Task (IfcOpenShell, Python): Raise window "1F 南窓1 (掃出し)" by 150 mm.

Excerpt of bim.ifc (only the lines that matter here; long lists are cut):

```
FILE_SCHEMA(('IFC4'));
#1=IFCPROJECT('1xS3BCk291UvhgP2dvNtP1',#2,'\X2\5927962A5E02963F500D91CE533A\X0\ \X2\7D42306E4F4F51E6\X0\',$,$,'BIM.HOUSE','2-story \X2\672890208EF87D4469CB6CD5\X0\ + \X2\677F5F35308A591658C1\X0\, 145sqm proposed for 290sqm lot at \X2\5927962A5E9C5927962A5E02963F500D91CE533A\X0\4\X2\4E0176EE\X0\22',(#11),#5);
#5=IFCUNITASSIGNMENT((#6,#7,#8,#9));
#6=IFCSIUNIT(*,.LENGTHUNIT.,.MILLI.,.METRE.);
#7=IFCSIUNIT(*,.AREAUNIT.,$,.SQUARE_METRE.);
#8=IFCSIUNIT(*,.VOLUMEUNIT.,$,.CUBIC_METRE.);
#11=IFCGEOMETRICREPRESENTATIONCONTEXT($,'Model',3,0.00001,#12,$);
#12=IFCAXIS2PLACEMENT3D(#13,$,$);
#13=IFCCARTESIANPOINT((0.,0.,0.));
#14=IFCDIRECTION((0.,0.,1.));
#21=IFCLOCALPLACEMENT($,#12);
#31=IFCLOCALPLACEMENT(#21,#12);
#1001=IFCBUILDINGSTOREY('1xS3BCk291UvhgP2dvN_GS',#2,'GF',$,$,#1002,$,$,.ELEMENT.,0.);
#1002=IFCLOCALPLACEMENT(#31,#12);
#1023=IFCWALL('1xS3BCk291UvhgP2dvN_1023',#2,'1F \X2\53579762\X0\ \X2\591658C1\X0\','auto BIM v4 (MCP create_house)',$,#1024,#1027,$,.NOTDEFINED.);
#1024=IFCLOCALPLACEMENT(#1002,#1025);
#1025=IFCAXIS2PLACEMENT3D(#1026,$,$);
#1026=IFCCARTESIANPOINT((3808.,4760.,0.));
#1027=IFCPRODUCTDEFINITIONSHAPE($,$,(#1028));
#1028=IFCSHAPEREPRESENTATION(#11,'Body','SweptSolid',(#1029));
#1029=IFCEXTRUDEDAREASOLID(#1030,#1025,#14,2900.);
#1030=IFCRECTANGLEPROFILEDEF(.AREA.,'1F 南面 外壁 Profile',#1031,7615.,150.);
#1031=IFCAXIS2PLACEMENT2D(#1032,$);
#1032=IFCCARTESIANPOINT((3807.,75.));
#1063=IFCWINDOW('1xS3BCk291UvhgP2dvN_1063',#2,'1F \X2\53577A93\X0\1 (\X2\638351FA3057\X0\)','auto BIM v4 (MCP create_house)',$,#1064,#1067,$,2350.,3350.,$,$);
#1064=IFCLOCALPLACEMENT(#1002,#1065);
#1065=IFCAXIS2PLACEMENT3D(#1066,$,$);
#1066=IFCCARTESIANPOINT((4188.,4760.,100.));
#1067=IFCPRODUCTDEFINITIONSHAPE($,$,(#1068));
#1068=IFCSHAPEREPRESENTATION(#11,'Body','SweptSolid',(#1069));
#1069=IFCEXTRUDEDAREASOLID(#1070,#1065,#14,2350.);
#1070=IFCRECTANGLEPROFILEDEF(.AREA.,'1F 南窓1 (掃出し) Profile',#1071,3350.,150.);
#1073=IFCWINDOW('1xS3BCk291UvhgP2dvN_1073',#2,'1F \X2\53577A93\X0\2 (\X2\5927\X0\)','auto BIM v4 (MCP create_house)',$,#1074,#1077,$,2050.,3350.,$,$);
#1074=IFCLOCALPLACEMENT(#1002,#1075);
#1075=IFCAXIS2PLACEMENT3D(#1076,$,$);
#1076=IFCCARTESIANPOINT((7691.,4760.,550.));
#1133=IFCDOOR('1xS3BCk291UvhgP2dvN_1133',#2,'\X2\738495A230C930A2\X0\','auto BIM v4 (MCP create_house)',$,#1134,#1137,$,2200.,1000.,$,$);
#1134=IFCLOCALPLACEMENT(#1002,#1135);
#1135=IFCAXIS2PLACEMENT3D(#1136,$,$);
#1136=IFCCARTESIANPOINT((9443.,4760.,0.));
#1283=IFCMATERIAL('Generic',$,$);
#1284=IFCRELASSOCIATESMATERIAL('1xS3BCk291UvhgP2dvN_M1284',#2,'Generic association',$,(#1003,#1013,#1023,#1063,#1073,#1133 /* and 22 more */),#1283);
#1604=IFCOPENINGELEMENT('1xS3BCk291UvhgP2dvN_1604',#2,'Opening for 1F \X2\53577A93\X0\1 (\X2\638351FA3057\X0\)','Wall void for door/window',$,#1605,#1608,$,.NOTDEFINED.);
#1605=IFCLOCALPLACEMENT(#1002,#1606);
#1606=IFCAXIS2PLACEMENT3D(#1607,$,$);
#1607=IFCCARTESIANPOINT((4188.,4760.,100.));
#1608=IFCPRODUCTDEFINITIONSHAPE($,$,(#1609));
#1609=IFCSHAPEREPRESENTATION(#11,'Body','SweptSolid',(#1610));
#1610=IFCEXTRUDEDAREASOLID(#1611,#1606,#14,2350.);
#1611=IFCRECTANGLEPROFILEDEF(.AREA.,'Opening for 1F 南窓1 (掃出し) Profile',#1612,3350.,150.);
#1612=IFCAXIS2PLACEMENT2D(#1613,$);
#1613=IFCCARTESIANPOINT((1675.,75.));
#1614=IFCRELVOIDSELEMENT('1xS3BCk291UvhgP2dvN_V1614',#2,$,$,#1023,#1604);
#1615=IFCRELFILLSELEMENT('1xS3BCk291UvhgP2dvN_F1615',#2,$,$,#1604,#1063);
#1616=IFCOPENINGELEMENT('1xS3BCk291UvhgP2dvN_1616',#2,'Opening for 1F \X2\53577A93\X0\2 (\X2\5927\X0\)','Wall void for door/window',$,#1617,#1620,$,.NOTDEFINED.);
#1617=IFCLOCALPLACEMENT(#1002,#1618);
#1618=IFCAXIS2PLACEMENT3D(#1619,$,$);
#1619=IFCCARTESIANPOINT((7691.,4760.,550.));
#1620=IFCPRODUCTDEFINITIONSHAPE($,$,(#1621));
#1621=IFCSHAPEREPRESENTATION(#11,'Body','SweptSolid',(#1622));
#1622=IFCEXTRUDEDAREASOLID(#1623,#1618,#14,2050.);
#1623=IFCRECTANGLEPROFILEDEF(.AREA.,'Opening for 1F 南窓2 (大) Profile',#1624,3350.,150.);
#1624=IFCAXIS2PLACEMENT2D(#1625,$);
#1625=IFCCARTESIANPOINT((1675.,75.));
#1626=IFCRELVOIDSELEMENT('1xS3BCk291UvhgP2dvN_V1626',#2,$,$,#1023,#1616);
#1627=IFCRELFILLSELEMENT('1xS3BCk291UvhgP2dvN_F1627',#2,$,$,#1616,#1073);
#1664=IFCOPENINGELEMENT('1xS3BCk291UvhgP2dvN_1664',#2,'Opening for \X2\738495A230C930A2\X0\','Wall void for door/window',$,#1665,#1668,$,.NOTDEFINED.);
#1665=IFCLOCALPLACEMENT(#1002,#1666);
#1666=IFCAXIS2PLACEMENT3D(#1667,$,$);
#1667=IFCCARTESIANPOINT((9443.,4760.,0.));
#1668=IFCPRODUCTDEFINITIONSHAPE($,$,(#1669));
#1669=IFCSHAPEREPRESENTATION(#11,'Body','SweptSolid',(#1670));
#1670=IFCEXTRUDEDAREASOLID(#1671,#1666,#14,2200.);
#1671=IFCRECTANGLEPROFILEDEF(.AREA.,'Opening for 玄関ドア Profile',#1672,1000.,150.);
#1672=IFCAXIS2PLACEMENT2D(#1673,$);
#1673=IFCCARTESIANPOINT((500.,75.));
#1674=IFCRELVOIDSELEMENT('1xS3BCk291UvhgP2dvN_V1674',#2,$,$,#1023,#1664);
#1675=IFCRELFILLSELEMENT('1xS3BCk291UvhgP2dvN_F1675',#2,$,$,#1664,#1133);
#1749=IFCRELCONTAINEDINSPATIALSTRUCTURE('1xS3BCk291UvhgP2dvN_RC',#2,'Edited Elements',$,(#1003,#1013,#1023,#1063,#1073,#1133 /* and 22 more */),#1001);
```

```python
import numpy as np
import ifcopenshell
import ifcopenshell.api.geometry
import ifcopenshell.util.placement
import ifcopenshell.util.unit

model = ifcopenshell.open("bim.ifc")
unit_scale = ifcopenshell.util.unit.calculate_unit_scale(model)

window = model.by_id(1063)
opening = window.FillsVoids[0].RelatingOpeningElement
dz = 150.0

shift = np.array([0.0, 0.0, dz])
# The window is not placed relative to its opening, so move both.
for product in (opening, window):
    matrix = ifcopenshell.util.placement.get_local_placement(product.ObjectPlacement)
    matrix[:3, 3] += shift
    ifcopenshell.api.geometry.edit_object_placement(model, product=product, matrix=matrix, is_si=False)

print(f"moved by {dz * unit_scale:+.3f} m")

model.write("bim_edited.ifc")
```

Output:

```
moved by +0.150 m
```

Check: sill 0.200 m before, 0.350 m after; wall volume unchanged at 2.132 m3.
